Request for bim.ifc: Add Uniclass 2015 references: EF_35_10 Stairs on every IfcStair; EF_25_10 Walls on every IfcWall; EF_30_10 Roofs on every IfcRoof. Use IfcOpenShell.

First a look at what the model holds.

```python
import ifcopenshell

model = ifcopenshell.open("bim.ifc")
print(model.schema)
print("classifications:", [c.Name for c in model.by_type("IfcClassification")])
for ifc_class in ("IfcDoor", "IfcRoof", "IfcStair", "IfcWall", "IfcWindow"):
    print(ifc_class, len(model.by_type(ifc_class)))
```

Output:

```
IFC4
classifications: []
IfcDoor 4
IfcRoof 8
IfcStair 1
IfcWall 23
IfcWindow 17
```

```python
import ifcopenshell
import ifcopenshell.api.classification

model = ifcopenshell.open("bim.ifc")

system = ifcopenshell.api.classification.add_classification(model, classification="Uniclass 2015")

codes = {
    "IfcStair": ("EF_35_10", "Stairs"),
    "IfcWall": ("EF_25_10", "Walls"),
    "IfcRoof": ("EF_30_10", "Roofs"),
}
for ifc_class, (code, name) in codes.items():
    products = model.by_type(ifc_class)
    ifcopenshell.api.classification.add_reference(
        model, products=products, classification=system, identification=code, name=name
    )
    print(code, len(products))

model.write("bim_updated.ifc")
```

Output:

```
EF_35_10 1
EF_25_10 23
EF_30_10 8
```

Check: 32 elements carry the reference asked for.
